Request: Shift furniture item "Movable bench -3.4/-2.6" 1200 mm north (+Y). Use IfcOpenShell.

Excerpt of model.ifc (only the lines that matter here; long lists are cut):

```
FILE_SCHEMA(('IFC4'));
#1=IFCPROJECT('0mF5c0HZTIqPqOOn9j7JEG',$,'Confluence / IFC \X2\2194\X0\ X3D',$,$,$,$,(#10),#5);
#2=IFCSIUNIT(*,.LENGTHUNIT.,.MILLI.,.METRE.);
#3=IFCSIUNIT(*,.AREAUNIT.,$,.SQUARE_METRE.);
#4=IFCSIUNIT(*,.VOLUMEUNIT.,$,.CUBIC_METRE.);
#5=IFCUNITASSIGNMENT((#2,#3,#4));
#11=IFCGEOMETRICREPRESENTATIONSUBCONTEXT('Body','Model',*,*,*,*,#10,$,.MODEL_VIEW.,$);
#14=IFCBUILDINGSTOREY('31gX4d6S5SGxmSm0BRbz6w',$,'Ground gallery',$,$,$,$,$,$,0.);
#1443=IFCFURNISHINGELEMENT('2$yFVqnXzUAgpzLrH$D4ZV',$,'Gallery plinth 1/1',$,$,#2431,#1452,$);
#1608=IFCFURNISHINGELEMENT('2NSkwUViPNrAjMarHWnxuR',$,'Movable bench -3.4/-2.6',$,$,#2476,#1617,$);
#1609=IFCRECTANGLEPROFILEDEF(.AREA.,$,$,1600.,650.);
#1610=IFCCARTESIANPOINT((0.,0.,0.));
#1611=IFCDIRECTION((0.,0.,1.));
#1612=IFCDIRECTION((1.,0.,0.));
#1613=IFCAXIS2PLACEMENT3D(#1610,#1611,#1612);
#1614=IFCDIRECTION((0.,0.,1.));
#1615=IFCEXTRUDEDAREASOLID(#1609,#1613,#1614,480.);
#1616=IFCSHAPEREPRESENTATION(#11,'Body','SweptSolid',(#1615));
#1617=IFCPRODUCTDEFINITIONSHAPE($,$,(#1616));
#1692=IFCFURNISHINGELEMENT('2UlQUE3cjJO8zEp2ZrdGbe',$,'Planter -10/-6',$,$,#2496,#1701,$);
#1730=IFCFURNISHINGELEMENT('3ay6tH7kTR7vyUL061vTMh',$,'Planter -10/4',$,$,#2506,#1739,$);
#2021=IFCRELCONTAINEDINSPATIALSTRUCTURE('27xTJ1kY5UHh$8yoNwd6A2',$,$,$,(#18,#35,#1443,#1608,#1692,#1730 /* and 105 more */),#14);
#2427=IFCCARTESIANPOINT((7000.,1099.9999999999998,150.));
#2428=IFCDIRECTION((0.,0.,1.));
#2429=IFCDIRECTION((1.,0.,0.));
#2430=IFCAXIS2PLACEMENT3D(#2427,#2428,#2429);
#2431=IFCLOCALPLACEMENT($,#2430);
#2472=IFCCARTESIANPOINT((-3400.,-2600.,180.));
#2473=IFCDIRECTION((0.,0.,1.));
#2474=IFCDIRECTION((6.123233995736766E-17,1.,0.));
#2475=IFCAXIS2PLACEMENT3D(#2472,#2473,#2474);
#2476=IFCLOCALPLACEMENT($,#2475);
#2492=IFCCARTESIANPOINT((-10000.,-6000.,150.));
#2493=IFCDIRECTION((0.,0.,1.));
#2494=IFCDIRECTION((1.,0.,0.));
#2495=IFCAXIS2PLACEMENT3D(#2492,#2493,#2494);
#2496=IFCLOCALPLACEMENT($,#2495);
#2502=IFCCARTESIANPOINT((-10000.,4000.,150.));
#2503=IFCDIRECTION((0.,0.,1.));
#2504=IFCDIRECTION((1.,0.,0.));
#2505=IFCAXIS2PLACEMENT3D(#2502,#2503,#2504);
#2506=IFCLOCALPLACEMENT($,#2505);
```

```python
import ifcopenshell
import ifcopenshell.api.geometry
import ifcopenshell.util.placement
import ifcopenshell.util.unit

model = ifcopenshell.open("model.ifc")
unit_scale = ifcopenshell.util.unit.calculate_unit_scale(model)

item = model.by_id(1608)
matrix = ifcopenshell.util.placement.get_local_placement(item.ObjectPlacement)
matrix[1, 3] += 1.2 / unit_scale
ifcopenshell.api.geometry.edit_object_placement(model, product=item, matrix=matrix, is_si=False)

print(ifcopenshell.util.placement.get_local_placement(item.ObjectPlacement).round(3) + 0.0)

model.write("model_edited.ifc")
```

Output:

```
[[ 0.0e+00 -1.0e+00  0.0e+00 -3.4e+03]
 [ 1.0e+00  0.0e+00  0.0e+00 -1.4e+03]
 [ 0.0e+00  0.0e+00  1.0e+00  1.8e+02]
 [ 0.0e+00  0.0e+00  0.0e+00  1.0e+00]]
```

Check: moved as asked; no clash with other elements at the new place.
